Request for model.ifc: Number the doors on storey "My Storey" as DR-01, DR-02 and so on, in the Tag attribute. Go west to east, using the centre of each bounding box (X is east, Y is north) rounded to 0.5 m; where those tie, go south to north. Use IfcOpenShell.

First a look at what the model holds.

```python
import ifcopenshell
import ifcopenshell.util.element
import ifcopenshell.util.placement

model = ifcopenshell.open("model.ifc")
print(model.schema)
storey = next(s for s in model.by_type("IfcBuildingStorey") if s.Name == "My Storey")
doors = [e for e in ifcopenshell.util.element.get_decomposition(storey) if e.is_a("IfcDoor")]
for e in sorted(doors, key=lambda e: e.id()):
    origin = ifcopenshell.util.placement.get_local_placement(e.ObjectPlacement)[:3, 3]
    print(e.id(), e.Tag, e.Name, origin.round(2) + 0.0, sep=" | ")
```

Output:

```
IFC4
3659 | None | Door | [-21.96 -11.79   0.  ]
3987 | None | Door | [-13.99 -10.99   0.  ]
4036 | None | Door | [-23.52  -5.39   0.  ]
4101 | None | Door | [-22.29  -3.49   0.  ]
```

```python
import ifcopenshell
import ifcopenshell.geom
import ifcopenshell.util.element
import ifcopenshell.util.shape

model = ifcopenshell.open("model.ifc")
settings = ifcopenshell.geom.settings()
settings.set("use-world-coords", True)


def centre(element):
    shape = ifcopenshell.geom.create_shape(settings, element)
    return ifcopenshell.util.shape.get_bbox_centroid(shape.geometry)


storey = next(s for s in model.by_type("IfcBuildingStorey") if s.Name == "My Storey")
doors = [e for e in ifcopenshell.util.element.get_decomposition(storey) if e.is_a("IfcDoor")]

# Insertion points can sit at a corner or the storey origin, so sort by the geometry (in metres).
centres = {e: centre(e) for e in doors}
doors.sort(key=lambda e: (round(centres[e][0] / 0.5), centres[e][1]))

for i, e in enumerate(doors, start=1):
    number = f"DR-{i:02d}"
    e.Tag = number
    print(e.id(), number)

model.write("model_updated.ifc")
```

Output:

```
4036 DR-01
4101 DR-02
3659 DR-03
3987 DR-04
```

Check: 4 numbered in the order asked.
